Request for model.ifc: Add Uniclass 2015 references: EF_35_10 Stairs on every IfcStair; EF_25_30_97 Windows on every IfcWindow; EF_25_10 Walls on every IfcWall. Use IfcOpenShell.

First a look at what the model holds.

```python
import ifcopenshell

model = ifcopenshell.open("model.ifc")
print(model.schema)
print("classifications:", [c.Name for c in model.by_type("IfcClassification")])
for ifc_class in ("IfcDoor", "IfcRoof", "IfcStair", "IfcWall", "IfcWindow"):
    print(ifc_class, len(model.by_type(ifc_class)))
```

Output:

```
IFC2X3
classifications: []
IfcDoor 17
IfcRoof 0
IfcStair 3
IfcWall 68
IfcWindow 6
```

```python
import ifcopenshell
import ifcopenshell.api.classification

model = ifcopenshell.open("model.ifc")

# IFC2X3 requires Source and Edition and has no link from the project to the system.
system = model.create_entity("IfcClassification", Source="NBS", Edition="2015", Name="Uniclass 2015")

codes = {
    "IfcStair": ("EF_35_10", "Stairs"),
    "IfcWindow": ("EF_25_30_97", "Windows"),
    "IfcWall": ("EF_25_10", "Walls"),
}
for ifc_class, (code, name) in codes.items():
    products = model.by_type(ifc_class)
    ifcopenshell.api.classification.add_reference(
        model, products=products, classification=system, identification=code, name=name
    )
    print(code, len(products))

model.write("model_v2.ifc")
```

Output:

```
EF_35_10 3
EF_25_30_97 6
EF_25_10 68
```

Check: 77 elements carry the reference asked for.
